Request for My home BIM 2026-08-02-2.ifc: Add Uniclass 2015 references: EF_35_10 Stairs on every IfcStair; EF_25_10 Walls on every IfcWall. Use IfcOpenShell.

First a look at what the model holds.

```python
import ifcopenshell

model = ifcopenshell.open("My home BIM 2026-08-02-2.ifc")
print(model.schema)
print("classifications:", [c.Name for c in model.by_type("IfcClassification")])
for ifc_class in ("IfcDoor", "IfcRoof", "IfcStair", "IfcWall", "IfcWindow"):
    print(ifc_class, len(model.by_type(ifc_class)))
```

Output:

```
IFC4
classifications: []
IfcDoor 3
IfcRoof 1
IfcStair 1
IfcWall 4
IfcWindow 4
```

```python
import ifcopenshell
import ifcopenshell.api.classification

model = ifcopenshell.open("My home BIM 2026-08-02-2.ifc")

system = ifcopenshell.api.classification.add_classification(model, classification="Uniclass 2015")

codes = {
    "IfcStair": ("EF_35_10", "Stairs"),
    "IfcWall": ("EF_25_10", "Walls"),
}
for ifc_class, (code, name) in codes.items():
    products = model.by_type(ifc_class)
    ifcopenshell.api.classification.add_reference(
        model, products=products, classification=system, identification=code, name=name
    )
    print(code, len(products))

model.write("My home BIM 2026-08-02-2_rev.ifc")
```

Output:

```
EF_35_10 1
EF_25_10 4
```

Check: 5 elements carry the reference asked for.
